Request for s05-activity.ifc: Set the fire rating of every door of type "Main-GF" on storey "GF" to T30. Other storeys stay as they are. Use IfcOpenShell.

First a look at what the model holds.

```python
import ifcopenshell
import ifcopenshell.util.element

model = ifcopenshell.open("s05-activity.ifc")
print(model.schema)
storey = next(s for s in model.by_type("IfcBuildingStorey") if s.Name == "GF")
doors = [e for e in ifcopenshell.util.element.get_decomposition(storey) if e.is_a("IfcDoor")]
seen = {}
for e in doors:
    element_type = ifcopenshell.util.element.get_type(e)
    key = (element_type.Name if element_type != e and element_type else None, ifcopenshell.util.element.get_pset(e, "Pset_DoorCommon", "FireRating"))
    seen[key] = seen.get(key, 0) + 1
for (name, value), count in sorted(seen.items(), key=str):
    print(count, "x", name, "|", value)
```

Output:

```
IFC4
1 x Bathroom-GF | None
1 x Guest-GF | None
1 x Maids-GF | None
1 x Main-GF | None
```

```python
import ifcopenshell
import ifcopenshell.api.pset
import ifcopenshell.util.element

model = ifcopenshell.open("s05-activity.ifc")

storey = next(s for s in model.by_type("IfcBuildingStorey") if s.Name == "GF")
doors = [e for e in ifcopenshell.util.element.get_decomposition(storey) if e.is_a("IfcDoor")]

count = 0
for e in doors:
    element_type = ifcopenshell.util.element.get_type(e)
    if element_type in (None, e) or element_type.Name != "Main-GF":
        continue
    # add_pset returns the element's existing set when there is one.
    pset = ifcopenshell.api.pset.add_pset(model, product=e, name="Pset_DoorCommon")
    ifcopenshell.api.pset.edit_pset(model, pset=pset, properties={"FireRating": "T30"})
    count += 1

print(count, "doors updated")

model.write("s05-activity_v2.ifc")
```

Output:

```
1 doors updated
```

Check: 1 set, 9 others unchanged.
